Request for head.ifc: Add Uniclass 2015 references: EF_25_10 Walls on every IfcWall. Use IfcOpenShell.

First a look at what the model holds.

```python
import ifcopenshell

model = ifcopenshell.open("head.ifc")
print(model.schema)
print("classifications:", [c.Name for c in model.by_type("IfcClassification")])
for ifc_class in ("IfcDoor", "IfcRoof", "IfcStair", "IfcWall", "IfcWindow"):
    print(ifc_class, len(model.by_type(ifc_class)))
```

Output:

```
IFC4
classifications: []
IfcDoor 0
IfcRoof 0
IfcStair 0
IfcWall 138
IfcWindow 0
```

```python
import ifcopenshell
import ifcopenshell.api.classification

model = ifcopenshell.open("head.ifc")

system = ifcopenshell.api.classification.add_classification(model, classification="Uniclass 2015")

codes = {
    "IfcWall": ("EF_25_10", "Walls"),
}
for ifc_class, (code, name) in codes.items():
    products = model.by_type(ifc_class)
    ifcopenshell.api.classification.add_reference(
        model, products=products, classification=system, identification=code, name=name
    )
    print(code, len(products))

model.write("head-out.ifc")
```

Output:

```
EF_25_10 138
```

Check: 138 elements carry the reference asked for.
